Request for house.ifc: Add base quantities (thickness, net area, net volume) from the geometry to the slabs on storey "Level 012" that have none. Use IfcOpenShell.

First a look at what the model holds.

```python
import ifcopenshell
import ifcopenshell.util.element
import ifcopenshell.util.unit

model = ifcopenshell.open("house.ifc")
print(model.schema)
for unit_type in ("LENGTHUNIT", "AREAUNIT", "VOLUMEUNIT"):
    print(unit_type, ifcopenshell.util.unit.calculate_unit_scale(model, unit_type))
storey = next(s for s in model.by_type("IfcBuildingStorey") if s.Name == "Level 012")
slabs = [e for e in ifcopenshell.util.element.get_decomposition(storey) if e.is_a("IfcSlab")]
for e in sorted(slabs, key=lambda e: e.id()):
    print(e.id(), e.is_a(), e.Name, list(ifcopenshell.util.element.get_psets(e, qtos_only=True)), sep=" | ")
```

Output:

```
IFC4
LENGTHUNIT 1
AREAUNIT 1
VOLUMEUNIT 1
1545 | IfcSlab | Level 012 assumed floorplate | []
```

```python
import ifcopenshell
import ifcopenshell.api.pset
import ifcopenshell.geom
import ifcopenshell.util.element
import ifcopenshell.util.shape
import ifcopenshell.util.unit

model = ifcopenshell.open("house.ifc")
unit_scale = ifcopenshell.util.unit.calculate_unit_scale(model)
area_scale = ifcopenshell.util.unit.calculate_unit_scale(model, "AREAUNIT")
volume_scale = ifcopenshell.util.unit.calculate_unit_scale(model, "VOLUMEUNIT")
settings = ifcopenshell.geom.settings()

storey = next(s for s in model.by_type("IfcBuildingStorey") if s.Name == "Level 012")
slabs = [e for e in ifcopenshell.util.element.get_decomposition(storey) if e.is_a("IfcSlab")]

for e in sorted(slabs, key=lambda e: e.id()):
    if ifcopenshell.util.element.get_psets(e, qtos_only=True, should_inherit=False):
        continue
    # Geometry comes back in metres, in the element's own axes.
    shape = ifcopenshell.geom.create_shape(settings, e)
    values = {
        "Width": ifcopenshell.util.shape.get_z(shape.geometry) / unit_scale,
        "NetArea": ifcopenshell.util.shape.get_footprint_area(shape.geometry) / area_scale,
        "NetVolume": ifcopenshell.util.shape.get_volume(shape.geometry) / volume_scale,
    }
    qto = ifcopenshell.api.pset.add_qto(model, product=e, name="Qto_SlabBaseQuantities")
    ifcopenshell.api.pset.edit_qto(model, qto=qto, properties=values)
    print(e.id(), {k: round(v, 3) for k, v in values.items()})

model.write("house-out.ifc")
```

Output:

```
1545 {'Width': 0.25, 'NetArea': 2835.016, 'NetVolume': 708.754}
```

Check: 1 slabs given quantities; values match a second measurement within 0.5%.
